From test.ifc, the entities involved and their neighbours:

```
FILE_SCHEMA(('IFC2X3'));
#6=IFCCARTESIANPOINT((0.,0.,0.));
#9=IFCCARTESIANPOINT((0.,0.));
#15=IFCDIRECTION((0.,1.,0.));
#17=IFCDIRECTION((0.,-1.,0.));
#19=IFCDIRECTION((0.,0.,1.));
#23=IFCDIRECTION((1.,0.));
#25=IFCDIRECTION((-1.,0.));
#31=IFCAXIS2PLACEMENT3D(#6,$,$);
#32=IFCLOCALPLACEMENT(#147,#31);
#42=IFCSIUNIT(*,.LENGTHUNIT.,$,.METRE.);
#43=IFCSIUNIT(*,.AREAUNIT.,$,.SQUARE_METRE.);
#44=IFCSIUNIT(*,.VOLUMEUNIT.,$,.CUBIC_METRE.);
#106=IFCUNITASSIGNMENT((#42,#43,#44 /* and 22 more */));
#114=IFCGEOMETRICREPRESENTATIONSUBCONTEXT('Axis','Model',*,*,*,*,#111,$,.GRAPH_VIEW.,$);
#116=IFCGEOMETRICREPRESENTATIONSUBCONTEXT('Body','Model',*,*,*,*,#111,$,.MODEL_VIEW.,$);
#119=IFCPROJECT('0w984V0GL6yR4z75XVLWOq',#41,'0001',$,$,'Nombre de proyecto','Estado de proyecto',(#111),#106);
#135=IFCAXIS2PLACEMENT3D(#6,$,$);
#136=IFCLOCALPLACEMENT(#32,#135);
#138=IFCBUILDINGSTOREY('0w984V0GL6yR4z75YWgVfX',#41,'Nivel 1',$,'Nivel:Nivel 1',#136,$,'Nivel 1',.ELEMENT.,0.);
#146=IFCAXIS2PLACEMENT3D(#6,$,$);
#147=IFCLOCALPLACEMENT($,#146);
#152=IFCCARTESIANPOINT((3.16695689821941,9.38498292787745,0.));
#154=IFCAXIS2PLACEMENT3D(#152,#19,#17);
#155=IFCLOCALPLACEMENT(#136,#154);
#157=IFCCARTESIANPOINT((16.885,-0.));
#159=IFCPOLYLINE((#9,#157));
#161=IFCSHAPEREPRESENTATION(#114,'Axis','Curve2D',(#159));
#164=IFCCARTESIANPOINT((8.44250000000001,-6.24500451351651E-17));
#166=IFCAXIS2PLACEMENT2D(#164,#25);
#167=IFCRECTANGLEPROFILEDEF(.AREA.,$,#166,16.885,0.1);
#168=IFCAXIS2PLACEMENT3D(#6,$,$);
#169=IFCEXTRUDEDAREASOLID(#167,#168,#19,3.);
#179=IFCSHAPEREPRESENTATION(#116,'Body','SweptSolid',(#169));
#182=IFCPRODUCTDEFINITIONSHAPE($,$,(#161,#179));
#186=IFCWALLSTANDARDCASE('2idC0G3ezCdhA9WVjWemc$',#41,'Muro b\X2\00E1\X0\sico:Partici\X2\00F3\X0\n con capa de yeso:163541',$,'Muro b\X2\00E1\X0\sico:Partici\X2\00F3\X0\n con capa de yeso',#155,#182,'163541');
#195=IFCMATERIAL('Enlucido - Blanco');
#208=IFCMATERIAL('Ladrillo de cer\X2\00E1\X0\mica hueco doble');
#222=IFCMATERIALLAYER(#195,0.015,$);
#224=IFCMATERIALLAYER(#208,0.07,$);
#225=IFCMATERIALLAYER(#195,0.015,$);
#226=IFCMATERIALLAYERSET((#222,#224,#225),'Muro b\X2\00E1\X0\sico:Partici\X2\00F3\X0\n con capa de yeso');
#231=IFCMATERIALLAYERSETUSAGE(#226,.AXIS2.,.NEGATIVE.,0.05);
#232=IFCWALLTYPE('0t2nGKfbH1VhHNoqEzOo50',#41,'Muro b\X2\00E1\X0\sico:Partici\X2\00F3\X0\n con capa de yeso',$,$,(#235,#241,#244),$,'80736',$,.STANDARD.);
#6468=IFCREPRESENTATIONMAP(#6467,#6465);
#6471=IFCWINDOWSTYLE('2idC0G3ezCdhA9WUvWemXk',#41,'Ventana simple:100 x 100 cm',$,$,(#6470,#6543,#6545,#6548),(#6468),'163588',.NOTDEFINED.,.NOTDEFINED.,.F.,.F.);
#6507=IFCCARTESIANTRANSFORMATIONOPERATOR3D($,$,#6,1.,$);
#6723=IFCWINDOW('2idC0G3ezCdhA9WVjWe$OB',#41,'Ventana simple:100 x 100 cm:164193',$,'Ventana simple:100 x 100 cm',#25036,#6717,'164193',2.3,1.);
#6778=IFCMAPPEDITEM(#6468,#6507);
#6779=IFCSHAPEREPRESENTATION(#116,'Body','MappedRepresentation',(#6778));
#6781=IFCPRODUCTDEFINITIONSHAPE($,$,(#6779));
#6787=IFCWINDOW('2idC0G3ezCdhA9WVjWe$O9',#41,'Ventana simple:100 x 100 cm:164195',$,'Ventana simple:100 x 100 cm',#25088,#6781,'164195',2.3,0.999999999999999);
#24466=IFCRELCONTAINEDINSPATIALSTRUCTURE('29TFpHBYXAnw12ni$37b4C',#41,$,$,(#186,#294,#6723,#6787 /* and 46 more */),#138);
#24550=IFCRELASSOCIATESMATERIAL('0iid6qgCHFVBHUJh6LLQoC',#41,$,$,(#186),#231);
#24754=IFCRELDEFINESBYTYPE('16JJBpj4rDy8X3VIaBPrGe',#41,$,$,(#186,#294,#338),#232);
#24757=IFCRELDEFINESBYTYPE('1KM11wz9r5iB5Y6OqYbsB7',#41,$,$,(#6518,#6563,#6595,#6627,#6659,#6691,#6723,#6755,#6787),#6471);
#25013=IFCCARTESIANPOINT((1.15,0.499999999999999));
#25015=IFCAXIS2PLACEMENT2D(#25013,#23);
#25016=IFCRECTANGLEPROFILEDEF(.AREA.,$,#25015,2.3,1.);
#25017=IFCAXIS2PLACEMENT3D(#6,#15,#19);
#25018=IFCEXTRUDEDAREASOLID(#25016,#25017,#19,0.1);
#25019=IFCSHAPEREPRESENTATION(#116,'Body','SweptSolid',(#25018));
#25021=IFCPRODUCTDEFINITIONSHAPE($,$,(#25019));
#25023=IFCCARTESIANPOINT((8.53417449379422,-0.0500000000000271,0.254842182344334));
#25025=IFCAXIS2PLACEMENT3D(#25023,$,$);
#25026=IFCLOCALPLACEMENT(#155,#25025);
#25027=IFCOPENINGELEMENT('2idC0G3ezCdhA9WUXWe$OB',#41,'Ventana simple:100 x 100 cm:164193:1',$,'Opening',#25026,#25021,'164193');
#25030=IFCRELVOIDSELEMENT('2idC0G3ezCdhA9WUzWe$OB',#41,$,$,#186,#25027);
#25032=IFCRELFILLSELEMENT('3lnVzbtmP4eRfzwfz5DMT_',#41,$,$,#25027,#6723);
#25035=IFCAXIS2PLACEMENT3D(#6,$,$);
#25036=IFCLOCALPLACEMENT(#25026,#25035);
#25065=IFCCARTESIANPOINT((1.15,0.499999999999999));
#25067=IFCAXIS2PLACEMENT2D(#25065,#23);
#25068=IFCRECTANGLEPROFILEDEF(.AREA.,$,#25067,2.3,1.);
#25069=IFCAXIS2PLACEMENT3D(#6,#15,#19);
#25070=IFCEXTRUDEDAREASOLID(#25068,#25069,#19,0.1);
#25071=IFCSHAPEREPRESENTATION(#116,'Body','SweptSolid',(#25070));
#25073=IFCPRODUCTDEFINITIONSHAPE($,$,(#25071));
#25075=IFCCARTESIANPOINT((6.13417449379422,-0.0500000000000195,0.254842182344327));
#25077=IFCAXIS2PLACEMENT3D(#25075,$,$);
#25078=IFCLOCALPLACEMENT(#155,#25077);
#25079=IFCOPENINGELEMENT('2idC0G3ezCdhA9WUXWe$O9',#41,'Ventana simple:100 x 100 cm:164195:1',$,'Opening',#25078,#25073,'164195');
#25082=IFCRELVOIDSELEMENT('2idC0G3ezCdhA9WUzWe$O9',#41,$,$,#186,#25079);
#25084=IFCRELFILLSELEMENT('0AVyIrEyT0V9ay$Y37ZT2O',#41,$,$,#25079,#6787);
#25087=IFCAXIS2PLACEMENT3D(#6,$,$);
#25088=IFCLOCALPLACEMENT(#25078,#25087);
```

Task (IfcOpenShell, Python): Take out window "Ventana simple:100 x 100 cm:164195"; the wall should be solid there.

```python
import ifcopenshell
import ifcopenshell.api.feature
import ifcopenshell.api.root
import ifcopenshell.geom
import ifcopenshell.util.shape

model = ifcopenshell.open("test.ifc")
settings = ifcopenshell.geom.settings()


def volume(element):
    """Net volume in cubic metres, openings subtracted."""
    shape = ifcopenshell.geom.create_shape(settings, element)
    return ifcopenshell.util.shape.get_volume(shape.geometry)


window = model.by_guid("2idC0G3ezCdhA9WVjWe$O9")
opening = window.FillsVoids[0].RelatingOpeningElement
wall = opening.VoidsElements[0].RelatingBuildingElement
before = volume(wall)

ifcopenshell.api.root.remove_product(model, product=window)
ifcopenshell.api.feature.remove_feature(model, feature=opening)

after = volume(wall)

print(f"wall volume {before:.3f} -> {after:.3f} m3")

model.write("test_rev.ifc")
```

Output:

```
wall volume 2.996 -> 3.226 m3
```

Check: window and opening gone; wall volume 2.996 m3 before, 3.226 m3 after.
